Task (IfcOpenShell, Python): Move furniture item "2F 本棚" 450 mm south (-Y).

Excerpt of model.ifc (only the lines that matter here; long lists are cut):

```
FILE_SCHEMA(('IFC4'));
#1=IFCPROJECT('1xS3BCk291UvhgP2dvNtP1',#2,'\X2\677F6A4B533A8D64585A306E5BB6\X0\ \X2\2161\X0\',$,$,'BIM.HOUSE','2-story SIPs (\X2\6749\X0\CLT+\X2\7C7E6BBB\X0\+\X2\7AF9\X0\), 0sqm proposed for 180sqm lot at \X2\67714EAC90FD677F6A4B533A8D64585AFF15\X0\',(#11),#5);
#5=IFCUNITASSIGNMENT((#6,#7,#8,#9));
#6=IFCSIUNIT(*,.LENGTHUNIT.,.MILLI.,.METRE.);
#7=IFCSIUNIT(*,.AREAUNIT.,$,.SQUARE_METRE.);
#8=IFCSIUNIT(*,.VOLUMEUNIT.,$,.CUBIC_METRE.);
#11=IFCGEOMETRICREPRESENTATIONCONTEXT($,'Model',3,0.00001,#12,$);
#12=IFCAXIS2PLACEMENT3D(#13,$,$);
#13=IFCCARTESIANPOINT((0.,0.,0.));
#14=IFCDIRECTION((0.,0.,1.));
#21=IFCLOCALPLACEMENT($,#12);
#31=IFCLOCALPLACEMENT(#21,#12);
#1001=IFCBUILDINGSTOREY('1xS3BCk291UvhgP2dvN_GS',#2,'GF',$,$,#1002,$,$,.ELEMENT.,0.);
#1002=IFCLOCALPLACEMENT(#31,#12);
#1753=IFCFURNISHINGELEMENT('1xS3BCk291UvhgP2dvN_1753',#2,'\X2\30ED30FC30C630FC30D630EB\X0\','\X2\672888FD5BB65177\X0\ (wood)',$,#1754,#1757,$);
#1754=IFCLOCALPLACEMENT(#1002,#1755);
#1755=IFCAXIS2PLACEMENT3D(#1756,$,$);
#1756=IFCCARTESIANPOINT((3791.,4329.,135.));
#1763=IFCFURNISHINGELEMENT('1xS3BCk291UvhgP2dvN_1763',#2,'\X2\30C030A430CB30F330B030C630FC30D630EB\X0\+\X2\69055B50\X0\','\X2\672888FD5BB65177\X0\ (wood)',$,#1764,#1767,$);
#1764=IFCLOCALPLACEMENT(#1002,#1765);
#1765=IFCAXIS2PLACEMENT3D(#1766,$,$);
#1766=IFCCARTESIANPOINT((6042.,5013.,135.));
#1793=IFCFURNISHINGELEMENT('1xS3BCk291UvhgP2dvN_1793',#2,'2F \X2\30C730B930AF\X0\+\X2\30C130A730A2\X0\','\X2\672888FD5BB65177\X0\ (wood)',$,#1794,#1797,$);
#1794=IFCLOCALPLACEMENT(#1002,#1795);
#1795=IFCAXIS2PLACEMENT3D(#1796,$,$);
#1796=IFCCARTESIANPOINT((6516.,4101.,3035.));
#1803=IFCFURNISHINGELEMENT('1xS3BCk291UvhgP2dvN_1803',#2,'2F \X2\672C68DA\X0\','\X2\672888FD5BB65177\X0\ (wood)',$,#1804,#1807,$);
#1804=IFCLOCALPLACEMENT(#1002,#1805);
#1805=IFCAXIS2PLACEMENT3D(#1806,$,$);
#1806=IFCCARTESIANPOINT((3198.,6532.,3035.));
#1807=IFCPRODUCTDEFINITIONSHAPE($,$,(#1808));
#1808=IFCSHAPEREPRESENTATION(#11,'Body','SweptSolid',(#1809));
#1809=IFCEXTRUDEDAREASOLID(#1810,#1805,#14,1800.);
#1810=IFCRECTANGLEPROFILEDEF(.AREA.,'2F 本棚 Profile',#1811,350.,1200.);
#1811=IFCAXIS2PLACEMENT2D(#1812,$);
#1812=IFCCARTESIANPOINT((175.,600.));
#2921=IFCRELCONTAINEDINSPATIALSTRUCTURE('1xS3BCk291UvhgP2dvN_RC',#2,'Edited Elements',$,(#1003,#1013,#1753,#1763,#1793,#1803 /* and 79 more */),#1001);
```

```python
import ifcopenshell
import ifcopenshell.api.geometry
import ifcopenshell.util.placement
import ifcopenshell.util.unit

model = ifcopenshell.open("model.ifc")
unit_scale = ifcopenshell.util.unit.calculate_unit_scale(model)

item = model.by_id(1803)
matrix = ifcopenshell.util.placement.get_local_placement(item.ObjectPlacement)
matrix[1, 3] -= 0.45 / unit_scale
ifcopenshell.api.geometry.edit_object_placement(model, product=item, matrix=matrix, is_si=False)

print(ifcopenshell.util.placement.get_local_placement(item.ObjectPlacement).round(3) + 0.0)

model.write("model_updated.ifc")
```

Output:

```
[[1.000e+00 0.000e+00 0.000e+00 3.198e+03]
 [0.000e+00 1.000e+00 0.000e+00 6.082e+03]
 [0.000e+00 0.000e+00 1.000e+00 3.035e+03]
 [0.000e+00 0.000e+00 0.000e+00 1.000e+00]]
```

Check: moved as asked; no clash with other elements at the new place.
